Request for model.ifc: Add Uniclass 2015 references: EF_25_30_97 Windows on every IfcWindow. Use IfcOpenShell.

First a look at what the model holds.

```python
import ifcopenshell

model = ifcopenshell.open("model.ifc")
print(model.schema)
print("classifications:", [c.Name for c in model.by_type("IfcClassification")])
for ifc_class in ("IfcDoor", "IfcRoof", "IfcStair", "IfcWall", "IfcWindow"):
    print(ifc_class, len(model.by_type(ifc_class)))
```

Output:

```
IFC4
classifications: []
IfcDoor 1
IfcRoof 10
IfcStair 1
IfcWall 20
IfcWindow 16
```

```python
import ifcopenshell
import ifcopenshell.api.classification

model = ifcopenshell.open("model.ifc")

system = ifcopenshell.api.classification.add_classification(model, classification="Uniclass 2015")

codes = {
    "IfcWindow": ("EF_25_30_97", "Windows"),
}
for ifc_class, (code, name) in codes.items():
    products = model.by_type(ifc_class)
    ifcopenshell.api.classification.add_reference(
        model, products=products, classification=system, identification=code, name=name
    )
    print(code, len(products))

model.write("model_edited.ifc")
```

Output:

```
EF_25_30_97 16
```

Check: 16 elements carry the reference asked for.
